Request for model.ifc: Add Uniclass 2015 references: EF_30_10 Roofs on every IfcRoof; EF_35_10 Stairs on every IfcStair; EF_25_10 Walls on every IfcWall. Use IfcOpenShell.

First a look at what the model holds.

```python
import ifcopenshell

model = ifcopenshell.open("model.ifc")
print(model.schema)
print("classifications:", [c.Name for c in model.by_type("IfcClassification")])
for ifc_class in ("IfcDoor", "IfcRoof", "IfcStair", "IfcWall", "IfcWindow"):
    print(ifc_class, len(model.by_type(ifc_class)))
```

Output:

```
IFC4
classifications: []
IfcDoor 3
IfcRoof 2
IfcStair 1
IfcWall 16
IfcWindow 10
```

```python
import ifcopenshell
import ifcopenshell.api.classification

model = ifcopenshell.open("model.ifc")

system = ifcopenshell.api.classification.add_classification(model, classification="Uniclass 2015")

codes = {
    "IfcRoof": ("EF_30_10", "Roofs"),
    "IfcStair": ("EF_35_10", "Stairs"),
    "IfcWall": ("EF_25_10", "Walls"),
}
for ifc_class, (code, name) in codes.items():
    products = model.by_type(ifc_class)
    ifcopenshell.api.classification.add_reference(
        model, products=products, classification=system, identification=code, name=name
    )
    print(code, len(products))

model.write("model-out.ifc")
```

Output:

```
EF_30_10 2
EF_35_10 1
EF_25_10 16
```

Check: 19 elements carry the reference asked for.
